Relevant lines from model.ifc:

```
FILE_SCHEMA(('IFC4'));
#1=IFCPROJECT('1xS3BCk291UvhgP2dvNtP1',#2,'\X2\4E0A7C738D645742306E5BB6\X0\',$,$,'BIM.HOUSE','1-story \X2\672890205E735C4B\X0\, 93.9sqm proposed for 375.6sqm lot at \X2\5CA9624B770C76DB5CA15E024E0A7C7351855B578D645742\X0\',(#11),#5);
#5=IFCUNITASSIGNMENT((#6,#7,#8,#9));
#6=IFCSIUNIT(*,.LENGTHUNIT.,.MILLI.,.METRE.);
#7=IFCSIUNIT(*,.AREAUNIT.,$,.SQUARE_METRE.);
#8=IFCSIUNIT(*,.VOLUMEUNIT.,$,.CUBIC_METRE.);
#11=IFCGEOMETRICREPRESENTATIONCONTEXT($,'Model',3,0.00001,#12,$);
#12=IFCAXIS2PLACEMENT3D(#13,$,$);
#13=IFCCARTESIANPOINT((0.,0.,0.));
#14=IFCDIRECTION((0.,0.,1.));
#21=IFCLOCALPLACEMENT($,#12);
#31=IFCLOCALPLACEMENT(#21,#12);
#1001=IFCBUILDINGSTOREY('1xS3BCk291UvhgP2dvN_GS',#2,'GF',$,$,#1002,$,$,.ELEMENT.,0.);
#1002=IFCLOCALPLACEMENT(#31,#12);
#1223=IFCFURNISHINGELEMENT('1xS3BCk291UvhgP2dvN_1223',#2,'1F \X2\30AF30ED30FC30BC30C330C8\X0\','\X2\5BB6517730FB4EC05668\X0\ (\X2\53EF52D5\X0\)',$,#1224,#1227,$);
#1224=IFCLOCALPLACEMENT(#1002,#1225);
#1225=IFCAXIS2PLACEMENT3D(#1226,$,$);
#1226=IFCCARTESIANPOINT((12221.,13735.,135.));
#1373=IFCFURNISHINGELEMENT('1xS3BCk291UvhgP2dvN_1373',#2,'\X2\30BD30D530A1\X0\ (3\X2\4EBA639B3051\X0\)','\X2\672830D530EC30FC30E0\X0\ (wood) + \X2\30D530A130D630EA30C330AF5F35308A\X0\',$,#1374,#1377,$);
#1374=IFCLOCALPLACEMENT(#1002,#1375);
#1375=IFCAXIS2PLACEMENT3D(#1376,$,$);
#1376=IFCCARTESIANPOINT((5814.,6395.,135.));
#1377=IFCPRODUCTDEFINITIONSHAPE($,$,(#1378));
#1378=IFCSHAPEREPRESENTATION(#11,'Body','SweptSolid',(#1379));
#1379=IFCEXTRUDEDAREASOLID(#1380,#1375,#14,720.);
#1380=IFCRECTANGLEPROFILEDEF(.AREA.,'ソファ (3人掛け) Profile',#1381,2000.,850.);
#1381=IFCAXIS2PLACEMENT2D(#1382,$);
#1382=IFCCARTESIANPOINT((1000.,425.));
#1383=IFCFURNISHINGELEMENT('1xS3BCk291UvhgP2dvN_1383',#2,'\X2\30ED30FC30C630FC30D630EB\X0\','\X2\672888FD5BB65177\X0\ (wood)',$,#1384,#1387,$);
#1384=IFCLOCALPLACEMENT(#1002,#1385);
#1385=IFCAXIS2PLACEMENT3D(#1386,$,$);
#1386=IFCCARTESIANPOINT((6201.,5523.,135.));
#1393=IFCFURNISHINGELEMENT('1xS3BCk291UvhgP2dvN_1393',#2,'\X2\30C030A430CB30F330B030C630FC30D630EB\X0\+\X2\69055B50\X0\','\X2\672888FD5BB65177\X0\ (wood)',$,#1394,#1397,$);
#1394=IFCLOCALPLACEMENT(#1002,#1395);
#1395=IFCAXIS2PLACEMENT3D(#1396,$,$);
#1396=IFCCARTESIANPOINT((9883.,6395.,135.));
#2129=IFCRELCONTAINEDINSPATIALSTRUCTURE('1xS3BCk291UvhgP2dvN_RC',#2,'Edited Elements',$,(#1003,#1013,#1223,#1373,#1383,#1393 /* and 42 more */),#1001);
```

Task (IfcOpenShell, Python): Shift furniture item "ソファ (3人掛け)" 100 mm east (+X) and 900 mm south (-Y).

```python
import ifcopenshell
import ifcopenshell.api.geometry
import ifcopenshell.util.placement
import ifcopenshell.util.unit

model = ifcopenshell.open("model.ifc")
unit_scale = ifcopenshell.util.unit.calculate_unit_scale(model)

item = model.by_guid("1xS3BCk291UvhgP2dvN_1373")
matrix = ifcopenshell.util.placement.get_local_placement(item.ObjectPlacement)
matrix[0, 3] += 0.1 / unit_scale
matrix[1, 3] -= 0.9 / unit_scale
ifcopenshell.api.geometry.edit_object_placement(model, product=item, matrix=matrix, is_si=False)

print(ifcopenshell.util.placement.get_local_placement(item.ObjectPlacement).round(3) + 0.0)

model.write("model-out.ifc")
```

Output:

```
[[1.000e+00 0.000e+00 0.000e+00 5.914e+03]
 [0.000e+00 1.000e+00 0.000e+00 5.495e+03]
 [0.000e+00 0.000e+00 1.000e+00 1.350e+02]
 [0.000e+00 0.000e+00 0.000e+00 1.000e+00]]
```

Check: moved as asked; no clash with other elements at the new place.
